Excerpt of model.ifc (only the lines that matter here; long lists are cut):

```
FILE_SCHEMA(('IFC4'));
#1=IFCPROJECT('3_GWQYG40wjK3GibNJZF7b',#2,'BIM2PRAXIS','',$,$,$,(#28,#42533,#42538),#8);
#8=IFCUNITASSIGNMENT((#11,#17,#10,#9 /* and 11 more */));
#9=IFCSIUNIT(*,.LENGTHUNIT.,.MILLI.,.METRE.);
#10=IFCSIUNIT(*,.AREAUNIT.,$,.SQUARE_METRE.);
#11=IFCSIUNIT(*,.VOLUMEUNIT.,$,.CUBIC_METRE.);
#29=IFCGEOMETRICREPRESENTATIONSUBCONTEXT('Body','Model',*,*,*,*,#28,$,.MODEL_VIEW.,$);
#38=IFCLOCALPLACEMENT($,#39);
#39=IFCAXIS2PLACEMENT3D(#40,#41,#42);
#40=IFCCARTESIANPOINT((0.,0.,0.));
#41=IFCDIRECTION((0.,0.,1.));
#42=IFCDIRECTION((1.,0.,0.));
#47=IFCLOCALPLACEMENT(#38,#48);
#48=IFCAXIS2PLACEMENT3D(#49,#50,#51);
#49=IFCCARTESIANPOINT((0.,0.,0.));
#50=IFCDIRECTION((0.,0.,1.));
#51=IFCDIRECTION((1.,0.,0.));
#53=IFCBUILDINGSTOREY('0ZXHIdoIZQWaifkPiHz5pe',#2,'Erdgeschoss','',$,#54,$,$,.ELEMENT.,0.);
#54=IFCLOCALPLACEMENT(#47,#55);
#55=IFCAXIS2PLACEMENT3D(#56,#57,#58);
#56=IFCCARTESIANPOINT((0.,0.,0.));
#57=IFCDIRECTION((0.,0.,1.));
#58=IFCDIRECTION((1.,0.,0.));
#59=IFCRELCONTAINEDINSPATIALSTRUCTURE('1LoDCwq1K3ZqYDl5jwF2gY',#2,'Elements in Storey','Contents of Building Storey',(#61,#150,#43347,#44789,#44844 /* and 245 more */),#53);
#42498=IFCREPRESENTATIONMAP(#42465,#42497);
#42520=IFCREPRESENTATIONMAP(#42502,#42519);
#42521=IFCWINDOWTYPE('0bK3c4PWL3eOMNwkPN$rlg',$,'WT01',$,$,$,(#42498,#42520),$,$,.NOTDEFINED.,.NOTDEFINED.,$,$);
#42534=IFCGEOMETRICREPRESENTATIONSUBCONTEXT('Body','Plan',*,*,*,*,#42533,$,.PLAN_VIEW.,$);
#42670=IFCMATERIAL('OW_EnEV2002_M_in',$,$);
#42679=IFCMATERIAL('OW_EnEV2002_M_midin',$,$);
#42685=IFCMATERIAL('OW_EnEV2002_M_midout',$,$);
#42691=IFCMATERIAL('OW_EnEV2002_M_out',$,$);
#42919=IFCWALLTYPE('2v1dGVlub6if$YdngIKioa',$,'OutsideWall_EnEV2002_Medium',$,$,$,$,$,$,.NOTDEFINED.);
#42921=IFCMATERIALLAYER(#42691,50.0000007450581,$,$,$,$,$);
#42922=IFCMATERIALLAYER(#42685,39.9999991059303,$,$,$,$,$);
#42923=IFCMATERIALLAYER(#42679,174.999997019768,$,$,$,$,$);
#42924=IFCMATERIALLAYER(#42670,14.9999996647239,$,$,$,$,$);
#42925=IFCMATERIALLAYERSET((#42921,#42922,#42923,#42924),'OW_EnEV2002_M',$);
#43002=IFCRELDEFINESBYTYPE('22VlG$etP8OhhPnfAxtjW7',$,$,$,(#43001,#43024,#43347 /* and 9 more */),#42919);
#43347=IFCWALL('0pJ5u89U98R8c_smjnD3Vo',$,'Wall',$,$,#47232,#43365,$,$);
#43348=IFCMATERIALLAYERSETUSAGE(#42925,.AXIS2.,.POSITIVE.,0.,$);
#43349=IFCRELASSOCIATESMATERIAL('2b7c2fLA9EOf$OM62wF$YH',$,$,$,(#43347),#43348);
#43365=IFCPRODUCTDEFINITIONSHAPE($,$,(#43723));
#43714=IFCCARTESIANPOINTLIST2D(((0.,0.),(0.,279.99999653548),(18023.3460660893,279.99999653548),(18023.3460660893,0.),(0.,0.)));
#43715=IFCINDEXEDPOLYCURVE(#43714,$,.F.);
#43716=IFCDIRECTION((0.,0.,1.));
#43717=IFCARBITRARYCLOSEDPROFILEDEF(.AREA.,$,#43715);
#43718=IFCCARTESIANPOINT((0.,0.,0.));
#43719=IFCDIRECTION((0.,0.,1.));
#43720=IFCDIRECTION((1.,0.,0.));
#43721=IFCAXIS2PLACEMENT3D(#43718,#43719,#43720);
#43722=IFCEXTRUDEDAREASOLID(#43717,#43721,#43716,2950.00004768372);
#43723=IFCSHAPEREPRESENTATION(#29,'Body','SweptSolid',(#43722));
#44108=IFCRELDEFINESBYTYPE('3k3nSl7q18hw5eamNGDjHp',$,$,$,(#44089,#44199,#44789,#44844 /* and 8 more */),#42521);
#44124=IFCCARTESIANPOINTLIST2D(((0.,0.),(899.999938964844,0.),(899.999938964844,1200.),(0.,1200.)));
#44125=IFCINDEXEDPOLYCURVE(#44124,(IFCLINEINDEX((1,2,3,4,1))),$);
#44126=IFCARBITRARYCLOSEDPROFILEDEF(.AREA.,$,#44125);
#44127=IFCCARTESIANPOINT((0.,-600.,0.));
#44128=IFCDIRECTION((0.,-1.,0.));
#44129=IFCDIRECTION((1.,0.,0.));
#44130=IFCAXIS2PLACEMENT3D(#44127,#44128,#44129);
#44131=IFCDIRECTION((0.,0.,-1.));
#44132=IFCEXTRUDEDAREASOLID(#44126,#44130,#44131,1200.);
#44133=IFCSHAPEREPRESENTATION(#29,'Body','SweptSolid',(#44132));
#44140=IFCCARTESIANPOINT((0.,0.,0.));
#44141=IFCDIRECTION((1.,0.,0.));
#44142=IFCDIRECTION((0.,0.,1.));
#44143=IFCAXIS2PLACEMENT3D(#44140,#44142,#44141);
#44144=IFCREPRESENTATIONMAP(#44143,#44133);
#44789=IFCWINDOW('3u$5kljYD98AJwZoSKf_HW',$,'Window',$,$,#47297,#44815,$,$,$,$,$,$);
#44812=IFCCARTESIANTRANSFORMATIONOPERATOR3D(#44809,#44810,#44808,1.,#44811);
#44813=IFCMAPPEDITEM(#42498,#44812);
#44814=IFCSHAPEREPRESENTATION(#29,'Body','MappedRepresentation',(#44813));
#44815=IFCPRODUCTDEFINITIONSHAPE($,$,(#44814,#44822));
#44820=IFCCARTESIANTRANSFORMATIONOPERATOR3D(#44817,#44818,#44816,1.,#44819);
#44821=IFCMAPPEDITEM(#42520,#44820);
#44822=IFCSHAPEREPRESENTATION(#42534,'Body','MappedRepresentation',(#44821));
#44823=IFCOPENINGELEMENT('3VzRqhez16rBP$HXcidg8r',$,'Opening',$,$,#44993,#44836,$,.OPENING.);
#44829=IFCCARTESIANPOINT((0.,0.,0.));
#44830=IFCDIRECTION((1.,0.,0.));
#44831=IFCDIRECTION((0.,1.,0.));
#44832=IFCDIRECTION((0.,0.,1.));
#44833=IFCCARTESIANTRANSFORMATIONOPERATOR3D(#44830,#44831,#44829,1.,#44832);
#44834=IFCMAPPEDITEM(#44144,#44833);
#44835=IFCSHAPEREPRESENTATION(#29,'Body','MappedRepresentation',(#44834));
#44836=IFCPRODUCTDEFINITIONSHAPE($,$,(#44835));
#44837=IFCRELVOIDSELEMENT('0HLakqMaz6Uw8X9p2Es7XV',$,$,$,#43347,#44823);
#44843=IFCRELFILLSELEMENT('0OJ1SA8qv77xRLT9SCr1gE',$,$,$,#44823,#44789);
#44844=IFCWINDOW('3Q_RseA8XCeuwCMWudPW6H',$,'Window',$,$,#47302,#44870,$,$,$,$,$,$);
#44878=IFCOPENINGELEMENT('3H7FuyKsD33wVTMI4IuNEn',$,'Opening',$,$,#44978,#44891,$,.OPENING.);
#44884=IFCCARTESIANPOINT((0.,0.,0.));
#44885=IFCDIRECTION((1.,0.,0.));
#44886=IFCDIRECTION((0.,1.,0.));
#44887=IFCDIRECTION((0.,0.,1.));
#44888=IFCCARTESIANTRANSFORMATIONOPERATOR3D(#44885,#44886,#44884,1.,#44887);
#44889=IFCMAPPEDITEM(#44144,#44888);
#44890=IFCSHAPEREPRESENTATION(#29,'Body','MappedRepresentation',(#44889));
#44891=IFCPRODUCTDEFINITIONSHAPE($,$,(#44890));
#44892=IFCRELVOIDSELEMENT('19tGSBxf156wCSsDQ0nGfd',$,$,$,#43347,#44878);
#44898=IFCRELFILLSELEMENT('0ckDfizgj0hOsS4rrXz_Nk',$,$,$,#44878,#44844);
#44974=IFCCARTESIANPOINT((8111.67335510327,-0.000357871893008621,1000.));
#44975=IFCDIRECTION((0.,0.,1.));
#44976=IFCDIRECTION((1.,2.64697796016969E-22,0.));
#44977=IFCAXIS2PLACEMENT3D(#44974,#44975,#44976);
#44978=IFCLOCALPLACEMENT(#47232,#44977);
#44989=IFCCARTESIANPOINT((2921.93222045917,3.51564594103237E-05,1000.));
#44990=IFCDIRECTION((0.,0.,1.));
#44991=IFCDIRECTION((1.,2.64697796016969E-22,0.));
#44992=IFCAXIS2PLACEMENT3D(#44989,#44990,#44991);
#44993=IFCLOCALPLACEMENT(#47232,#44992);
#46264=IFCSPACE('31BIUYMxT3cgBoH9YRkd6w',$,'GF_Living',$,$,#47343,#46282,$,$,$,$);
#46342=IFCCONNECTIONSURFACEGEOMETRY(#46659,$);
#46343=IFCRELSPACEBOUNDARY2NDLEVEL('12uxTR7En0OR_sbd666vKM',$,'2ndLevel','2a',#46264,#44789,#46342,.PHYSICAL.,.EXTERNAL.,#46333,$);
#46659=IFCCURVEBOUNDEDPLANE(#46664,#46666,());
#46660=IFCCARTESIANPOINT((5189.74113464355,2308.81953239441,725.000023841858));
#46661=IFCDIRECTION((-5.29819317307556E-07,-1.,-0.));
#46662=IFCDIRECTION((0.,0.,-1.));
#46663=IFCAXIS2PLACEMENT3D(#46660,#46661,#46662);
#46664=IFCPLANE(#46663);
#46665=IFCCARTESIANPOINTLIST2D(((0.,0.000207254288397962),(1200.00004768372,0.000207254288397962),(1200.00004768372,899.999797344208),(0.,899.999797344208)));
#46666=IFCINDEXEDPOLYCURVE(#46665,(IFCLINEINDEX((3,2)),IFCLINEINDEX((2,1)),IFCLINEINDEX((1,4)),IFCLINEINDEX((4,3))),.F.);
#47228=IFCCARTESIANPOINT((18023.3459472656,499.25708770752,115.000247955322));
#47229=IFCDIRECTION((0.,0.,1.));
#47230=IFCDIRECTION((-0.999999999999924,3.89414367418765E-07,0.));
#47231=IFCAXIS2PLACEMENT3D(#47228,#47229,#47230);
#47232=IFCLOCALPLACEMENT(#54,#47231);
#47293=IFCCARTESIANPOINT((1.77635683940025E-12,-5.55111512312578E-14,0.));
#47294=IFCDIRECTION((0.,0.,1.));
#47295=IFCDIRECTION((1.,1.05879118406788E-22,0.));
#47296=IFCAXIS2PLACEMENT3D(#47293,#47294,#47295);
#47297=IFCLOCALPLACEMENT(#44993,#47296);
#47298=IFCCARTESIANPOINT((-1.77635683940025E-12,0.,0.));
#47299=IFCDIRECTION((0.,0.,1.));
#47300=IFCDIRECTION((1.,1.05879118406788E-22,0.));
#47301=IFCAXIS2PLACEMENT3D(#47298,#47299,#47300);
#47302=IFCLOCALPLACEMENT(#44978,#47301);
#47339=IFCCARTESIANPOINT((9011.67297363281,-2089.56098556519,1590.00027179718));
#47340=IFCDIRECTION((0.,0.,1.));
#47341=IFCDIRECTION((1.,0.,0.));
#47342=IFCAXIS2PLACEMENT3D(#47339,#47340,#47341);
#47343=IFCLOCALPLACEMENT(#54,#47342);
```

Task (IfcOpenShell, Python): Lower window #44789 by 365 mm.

```python
import numpy as np
import ifcopenshell
import ifcopenshell.api.geometry
import ifcopenshell.util.placement
import ifcopenshell.util.unit

model = ifcopenshell.open("model.ifc")
unit_scale = ifcopenshell.util.unit.calculate_unit_scale(model)

window = model.by_id(44789)
opening = window.FillsVoids[0].RelatingOpeningElement
dz = -0.365 / unit_scale

shift = np.array([0.0, 0.0, dz])
# The window is placed relative to its opening, so it follows when the opening moves.
matrix = ifcopenshell.util.placement.get_local_placement(opening.ObjectPlacement)
matrix[:3, 3] += shift
ifcopenshell.api.geometry.edit_object_placement(
    model, product=opening, matrix=matrix, is_si=False, should_transform_children=True
)

# Space boundary surfaces are stored in each space's coordinates; move them too.
for rel in window.ProvidesBoundaries:
    if not rel.ConnectionGeometry:
        continue
    surface = rel.ConnectionGeometry.SurfaceOnRelatingElement.BasisSurface
    space_matrix = ifcopenshell.util.placement.get_local_placement(rel.RelatingSpace.ObjectPlacement)
    point = np.array(surface.Position.Location.Coordinates) + space_matrix[:3, :3].T @ shift
    surface.Position = model.createIfcAxis2Placement3D(
        model.createIfcCartesianPoint(point.tolist()), surface.Position.Axis, surface.Position.RefDirection
    )

print(f"moved by {dz * unit_scale:+.3f} m")

model.write("model_updated.ifc")
```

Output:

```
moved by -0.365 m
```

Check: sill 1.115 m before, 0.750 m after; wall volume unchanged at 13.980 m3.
